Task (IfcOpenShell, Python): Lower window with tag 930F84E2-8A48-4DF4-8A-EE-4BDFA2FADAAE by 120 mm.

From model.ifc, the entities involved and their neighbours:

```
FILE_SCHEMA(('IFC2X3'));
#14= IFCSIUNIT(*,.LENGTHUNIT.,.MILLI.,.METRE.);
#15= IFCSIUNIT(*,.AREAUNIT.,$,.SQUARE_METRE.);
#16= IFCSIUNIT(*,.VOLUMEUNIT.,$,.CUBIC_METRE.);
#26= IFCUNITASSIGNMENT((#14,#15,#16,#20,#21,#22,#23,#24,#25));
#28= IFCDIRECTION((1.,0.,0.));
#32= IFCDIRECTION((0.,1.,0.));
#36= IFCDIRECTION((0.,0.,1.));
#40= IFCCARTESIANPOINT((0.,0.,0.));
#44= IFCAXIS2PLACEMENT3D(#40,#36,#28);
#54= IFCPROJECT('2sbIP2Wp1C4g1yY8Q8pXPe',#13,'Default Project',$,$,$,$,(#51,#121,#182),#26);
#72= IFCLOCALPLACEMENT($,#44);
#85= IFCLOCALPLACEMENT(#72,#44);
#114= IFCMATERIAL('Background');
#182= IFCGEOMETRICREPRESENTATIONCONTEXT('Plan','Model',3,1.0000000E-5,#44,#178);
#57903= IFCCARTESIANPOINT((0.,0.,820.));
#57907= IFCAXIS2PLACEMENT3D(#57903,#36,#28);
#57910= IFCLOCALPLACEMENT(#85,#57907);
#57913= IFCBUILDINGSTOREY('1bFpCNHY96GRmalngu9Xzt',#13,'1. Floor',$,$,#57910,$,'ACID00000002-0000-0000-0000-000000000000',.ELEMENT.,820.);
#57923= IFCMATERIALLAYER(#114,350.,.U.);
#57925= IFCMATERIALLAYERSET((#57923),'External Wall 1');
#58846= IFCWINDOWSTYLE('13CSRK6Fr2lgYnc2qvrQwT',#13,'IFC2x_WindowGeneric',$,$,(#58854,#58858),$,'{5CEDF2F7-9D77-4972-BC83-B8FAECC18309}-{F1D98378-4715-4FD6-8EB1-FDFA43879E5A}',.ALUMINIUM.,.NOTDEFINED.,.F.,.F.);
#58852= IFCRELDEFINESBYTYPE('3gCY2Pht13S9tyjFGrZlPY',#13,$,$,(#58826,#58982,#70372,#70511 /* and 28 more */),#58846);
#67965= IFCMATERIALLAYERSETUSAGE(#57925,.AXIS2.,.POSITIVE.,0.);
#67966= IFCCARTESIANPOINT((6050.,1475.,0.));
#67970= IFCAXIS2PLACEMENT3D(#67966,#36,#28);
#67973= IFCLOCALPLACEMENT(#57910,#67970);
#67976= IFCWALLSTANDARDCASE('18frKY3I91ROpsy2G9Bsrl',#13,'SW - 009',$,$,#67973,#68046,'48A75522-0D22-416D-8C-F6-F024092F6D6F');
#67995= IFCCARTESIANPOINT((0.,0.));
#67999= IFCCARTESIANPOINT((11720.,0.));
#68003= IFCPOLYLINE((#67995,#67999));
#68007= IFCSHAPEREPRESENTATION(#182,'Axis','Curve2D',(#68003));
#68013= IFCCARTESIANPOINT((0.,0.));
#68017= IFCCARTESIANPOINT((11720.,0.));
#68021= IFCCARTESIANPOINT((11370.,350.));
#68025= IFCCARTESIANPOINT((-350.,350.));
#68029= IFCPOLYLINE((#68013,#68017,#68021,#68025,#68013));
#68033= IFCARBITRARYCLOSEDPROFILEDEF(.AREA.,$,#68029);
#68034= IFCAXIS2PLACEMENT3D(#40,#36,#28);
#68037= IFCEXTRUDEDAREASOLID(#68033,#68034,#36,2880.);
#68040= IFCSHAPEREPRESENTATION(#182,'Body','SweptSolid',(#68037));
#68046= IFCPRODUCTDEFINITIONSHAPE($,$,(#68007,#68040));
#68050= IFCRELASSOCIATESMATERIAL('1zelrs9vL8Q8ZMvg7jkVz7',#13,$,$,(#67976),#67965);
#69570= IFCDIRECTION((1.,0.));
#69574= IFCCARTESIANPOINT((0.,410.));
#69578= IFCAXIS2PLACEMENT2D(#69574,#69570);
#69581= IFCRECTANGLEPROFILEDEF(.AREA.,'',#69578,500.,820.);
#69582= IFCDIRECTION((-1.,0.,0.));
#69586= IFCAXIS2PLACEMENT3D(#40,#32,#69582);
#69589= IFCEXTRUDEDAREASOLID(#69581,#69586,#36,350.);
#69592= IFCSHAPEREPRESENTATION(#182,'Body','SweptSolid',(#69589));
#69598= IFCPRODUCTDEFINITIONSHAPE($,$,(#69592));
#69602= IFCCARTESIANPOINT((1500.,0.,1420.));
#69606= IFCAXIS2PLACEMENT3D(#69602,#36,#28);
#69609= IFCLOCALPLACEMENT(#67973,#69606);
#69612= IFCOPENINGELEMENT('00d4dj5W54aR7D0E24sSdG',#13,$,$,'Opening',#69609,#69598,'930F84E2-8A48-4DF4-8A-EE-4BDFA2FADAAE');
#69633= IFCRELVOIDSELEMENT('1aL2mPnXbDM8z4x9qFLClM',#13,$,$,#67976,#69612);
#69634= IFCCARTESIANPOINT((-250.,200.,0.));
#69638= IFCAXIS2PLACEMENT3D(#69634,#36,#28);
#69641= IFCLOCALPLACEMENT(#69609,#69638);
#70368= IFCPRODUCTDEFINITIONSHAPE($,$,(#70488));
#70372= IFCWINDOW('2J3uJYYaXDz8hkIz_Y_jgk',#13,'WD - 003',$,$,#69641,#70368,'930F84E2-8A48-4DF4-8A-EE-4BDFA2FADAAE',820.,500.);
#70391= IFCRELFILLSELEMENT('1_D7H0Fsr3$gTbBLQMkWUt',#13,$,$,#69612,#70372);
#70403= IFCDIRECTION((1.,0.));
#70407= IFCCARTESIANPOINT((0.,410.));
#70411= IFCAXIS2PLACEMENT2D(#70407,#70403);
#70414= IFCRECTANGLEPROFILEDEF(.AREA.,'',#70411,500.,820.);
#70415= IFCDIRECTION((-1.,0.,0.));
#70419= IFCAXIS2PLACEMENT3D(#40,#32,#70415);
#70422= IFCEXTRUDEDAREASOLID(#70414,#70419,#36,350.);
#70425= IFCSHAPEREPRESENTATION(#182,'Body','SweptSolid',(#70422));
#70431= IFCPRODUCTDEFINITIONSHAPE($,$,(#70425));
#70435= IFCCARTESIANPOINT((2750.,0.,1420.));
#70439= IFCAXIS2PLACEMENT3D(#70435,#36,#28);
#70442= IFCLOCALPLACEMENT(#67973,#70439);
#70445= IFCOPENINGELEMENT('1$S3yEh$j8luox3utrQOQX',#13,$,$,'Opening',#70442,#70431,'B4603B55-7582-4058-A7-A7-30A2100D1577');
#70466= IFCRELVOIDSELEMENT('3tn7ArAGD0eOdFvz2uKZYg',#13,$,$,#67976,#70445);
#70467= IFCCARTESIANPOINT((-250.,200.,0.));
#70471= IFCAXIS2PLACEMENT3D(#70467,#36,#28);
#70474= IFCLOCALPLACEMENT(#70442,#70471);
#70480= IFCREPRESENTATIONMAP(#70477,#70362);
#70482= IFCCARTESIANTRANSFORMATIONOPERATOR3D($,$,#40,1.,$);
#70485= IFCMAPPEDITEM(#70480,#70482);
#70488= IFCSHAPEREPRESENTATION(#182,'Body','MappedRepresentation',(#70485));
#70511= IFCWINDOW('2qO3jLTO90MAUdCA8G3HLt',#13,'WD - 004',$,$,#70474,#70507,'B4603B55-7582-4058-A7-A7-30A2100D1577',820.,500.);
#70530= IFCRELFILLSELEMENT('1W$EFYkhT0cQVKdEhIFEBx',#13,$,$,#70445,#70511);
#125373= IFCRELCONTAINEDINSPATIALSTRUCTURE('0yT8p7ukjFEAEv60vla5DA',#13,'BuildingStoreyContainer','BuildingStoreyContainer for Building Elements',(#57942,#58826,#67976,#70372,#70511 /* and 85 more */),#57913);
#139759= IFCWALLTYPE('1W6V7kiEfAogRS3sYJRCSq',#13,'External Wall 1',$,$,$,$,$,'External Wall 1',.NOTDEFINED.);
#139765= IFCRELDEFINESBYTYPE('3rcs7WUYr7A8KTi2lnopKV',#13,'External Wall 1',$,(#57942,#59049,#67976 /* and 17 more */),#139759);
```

```python
import numpy as np
import ifcopenshell
import ifcopenshell.api.geometry
import ifcopenshell.util.placement
import ifcopenshell.util.unit

model = ifcopenshell.open("model.ifc")
unit_scale = ifcopenshell.util.unit.calculate_unit_scale(model)

window = model.by_id(70372)
opening = window.FillsVoids[0].RelatingOpeningElement
dz = -0.12 / unit_scale

shift = np.array([0.0, 0.0, dz])
# The window is placed relative to its opening, so it follows when the opening moves.
matrix = ifcopenshell.util.placement.get_local_placement(opening.ObjectPlacement)
matrix[:3, 3] += shift
ifcopenshell.api.geometry.edit_object_placement(
    model, product=opening, matrix=matrix, is_si=False, should_transform_children=True
)

print(f"moved by {dz * unit_scale:+.3f} m")

model.write("model_updated.ifc")
```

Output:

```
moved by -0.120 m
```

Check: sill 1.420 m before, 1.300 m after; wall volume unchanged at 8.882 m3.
